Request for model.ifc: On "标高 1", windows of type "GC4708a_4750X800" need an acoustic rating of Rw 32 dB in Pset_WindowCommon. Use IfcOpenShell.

First a look at what the model holds.

```python
import ifcopenshell
import ifcopenshell.util.element

model = ifcopenshell.open("model.ifc")
print(model.schema)
storey = next(s for s in model.by_type("IfcBuildingStorey") if s.Name == "标高 1")
windows = [e for e in ifcopenshell.util.element.get_decomposition(storey) if e.is_a("IfcWindow")]
seen = {}
for e in windows:
    element_type = ifcopenshell.util.element.get_type(e)
    key = (element_type.Name if element_type != e and element_type else None, ifcopenshell.util.element.get_pset(e, "Pset_WindowCommon", "AcousticRating"))
    seen[key] = seen.get(key, 0) + 1
for (name, value), count in sorted(seen.items(), key=str):
    print(count, "x", name, "|", value)
```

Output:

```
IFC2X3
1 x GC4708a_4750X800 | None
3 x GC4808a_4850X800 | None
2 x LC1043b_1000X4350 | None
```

```python
import ifcopenshell
import ifcopenshell.api.pset
import ifcopenshell.util.element

model = ifcopenshell.open("model.ifc")

storey = next(s for s in model.by_type("IfcBuildingStorey") if s.Name == "标高 1")
windows = [e for e in ifcopenshell.util.element.get_decomposition(storey) if e.is_a("IfcWindow")]

count = 0
for e in windows:
    element_type = ifcopenshell.util.element.get_type(e)
    if element_type in (None, e) or element_type.Name != "GC4708a_4750X800":
        continue
    # add_pset returns the element's existing set when there is one.
    pset = ifcopenshell.api.pset.add_pset(model, product=e, name="Pset_WindowCommon")
    ifcopenshell.api.pset.edit_pset(model, pset=pset, properties={"AcousticRating": "Rw 32 dB"})
    count += 1

print(count, "windows updated")

model.write("model_v2.ifc")
```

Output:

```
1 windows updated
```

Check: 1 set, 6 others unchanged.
